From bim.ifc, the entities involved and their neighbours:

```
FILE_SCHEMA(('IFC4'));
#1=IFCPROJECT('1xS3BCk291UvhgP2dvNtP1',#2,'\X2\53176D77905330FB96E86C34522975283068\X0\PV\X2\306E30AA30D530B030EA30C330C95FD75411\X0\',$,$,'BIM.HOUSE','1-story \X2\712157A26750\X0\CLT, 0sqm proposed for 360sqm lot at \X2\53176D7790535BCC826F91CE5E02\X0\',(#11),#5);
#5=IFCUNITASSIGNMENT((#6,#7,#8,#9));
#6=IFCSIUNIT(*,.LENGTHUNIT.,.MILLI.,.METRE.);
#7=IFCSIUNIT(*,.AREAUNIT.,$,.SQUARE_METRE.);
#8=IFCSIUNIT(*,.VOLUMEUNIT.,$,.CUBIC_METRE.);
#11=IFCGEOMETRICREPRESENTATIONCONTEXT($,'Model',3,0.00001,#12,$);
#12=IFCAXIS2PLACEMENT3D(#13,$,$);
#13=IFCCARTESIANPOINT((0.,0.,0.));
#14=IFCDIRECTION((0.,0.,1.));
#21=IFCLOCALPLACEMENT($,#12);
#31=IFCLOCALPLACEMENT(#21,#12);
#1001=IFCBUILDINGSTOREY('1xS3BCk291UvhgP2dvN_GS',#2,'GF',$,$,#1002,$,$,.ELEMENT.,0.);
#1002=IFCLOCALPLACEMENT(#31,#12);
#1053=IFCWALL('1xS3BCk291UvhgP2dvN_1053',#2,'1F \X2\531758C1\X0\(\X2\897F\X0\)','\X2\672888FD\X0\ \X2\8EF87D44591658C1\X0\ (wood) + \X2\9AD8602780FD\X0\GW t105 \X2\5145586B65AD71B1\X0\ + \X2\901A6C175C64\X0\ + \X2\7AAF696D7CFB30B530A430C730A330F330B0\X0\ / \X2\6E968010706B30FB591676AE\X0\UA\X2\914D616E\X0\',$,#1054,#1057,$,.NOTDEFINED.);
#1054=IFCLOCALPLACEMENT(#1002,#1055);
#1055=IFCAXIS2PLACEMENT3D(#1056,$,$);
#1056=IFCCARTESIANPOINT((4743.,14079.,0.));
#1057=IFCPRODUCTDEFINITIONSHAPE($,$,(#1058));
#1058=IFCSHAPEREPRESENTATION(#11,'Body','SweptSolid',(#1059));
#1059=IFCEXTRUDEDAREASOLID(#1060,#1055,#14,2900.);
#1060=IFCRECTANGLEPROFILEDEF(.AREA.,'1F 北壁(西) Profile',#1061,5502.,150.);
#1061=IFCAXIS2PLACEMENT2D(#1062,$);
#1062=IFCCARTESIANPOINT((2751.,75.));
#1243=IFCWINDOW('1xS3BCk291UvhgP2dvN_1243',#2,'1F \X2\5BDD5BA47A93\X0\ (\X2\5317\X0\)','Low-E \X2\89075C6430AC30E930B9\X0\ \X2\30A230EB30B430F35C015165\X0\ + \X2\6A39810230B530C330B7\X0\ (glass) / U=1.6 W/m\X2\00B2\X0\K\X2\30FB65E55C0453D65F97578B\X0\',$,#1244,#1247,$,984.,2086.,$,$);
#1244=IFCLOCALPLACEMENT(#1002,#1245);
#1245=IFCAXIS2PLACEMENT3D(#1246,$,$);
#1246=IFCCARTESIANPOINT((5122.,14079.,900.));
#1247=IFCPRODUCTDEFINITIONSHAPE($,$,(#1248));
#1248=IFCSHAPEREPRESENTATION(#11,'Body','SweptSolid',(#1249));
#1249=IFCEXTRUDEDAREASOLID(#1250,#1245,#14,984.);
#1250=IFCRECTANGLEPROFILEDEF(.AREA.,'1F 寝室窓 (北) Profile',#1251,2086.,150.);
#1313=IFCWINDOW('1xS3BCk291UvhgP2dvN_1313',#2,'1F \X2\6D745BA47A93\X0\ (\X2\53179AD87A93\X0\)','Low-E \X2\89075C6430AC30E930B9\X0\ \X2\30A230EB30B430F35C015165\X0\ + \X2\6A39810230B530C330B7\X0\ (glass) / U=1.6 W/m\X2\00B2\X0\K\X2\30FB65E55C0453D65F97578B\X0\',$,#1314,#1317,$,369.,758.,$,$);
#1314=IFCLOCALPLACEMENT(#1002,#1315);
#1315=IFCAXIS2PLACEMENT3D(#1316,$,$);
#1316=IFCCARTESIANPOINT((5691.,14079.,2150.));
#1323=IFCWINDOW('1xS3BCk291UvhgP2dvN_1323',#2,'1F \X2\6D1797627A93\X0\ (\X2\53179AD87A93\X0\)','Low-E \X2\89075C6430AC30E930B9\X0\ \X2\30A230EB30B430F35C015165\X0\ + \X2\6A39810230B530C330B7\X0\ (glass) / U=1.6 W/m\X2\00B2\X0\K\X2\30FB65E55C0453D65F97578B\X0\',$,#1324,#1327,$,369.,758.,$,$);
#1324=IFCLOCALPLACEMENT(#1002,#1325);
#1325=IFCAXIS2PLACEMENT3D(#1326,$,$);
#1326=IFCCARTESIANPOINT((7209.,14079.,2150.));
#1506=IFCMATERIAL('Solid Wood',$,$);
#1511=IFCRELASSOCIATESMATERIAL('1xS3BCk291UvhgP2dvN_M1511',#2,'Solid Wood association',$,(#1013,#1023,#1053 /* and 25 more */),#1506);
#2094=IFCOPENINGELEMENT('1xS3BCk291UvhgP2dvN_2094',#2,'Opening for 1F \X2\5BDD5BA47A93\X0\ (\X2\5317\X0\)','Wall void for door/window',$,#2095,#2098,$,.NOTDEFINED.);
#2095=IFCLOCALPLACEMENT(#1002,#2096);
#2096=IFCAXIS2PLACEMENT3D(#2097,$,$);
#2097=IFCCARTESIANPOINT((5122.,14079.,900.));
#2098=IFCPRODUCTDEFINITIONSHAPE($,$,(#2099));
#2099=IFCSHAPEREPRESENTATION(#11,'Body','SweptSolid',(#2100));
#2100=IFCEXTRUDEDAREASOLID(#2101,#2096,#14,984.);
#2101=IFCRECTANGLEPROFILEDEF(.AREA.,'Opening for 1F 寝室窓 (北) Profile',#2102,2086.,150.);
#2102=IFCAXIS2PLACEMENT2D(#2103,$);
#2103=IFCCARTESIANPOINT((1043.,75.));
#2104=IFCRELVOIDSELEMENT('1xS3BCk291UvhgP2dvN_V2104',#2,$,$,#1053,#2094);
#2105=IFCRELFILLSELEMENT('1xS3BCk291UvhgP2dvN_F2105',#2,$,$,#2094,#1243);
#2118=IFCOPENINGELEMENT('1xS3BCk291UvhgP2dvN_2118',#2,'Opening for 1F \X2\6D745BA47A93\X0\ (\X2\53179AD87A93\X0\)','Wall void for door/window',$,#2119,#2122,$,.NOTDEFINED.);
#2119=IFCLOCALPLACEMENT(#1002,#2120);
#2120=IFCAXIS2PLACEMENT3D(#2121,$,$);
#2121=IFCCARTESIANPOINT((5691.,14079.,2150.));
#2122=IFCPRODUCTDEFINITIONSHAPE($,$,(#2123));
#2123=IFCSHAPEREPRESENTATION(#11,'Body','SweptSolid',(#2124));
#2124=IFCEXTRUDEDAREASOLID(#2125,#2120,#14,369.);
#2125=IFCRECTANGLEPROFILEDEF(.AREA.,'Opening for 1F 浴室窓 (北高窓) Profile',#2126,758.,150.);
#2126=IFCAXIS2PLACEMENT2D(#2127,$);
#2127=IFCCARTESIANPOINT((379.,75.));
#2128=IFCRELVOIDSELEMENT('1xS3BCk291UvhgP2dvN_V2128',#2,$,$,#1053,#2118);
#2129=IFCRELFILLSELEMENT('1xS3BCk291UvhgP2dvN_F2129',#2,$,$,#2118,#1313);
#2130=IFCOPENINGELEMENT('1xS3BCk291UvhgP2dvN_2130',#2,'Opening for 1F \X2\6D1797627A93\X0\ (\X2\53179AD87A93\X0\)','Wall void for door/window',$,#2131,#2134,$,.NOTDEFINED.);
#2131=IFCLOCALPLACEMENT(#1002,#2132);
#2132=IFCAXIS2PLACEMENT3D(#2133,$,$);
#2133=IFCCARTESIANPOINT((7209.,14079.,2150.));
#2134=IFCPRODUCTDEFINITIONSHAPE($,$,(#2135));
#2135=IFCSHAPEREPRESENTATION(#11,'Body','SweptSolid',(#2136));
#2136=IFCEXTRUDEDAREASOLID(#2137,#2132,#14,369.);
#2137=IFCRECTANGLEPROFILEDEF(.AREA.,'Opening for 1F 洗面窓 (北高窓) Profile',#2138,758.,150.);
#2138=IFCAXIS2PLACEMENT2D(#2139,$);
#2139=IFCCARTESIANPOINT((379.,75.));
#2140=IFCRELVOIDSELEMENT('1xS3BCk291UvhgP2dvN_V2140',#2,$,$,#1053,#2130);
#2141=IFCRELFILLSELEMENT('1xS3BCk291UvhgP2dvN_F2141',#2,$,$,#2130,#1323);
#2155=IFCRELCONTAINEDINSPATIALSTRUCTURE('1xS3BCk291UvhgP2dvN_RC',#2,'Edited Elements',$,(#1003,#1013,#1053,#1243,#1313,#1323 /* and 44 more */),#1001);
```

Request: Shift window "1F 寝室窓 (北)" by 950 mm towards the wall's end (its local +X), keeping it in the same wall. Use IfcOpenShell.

```python
import ifcopenshell
import ifcopenshell.api.geometry
import ifcopenshell.util.placement

model = ifcopenshell.open("bim.ifc")

window = model.by_guid("1xS3BCk291UvhgP2dvN_1243")
opening = window.FillsVoids[0].RelatingOpeningElement
wall = opening.VoidsElements[0].RelatingBuildingElement

wall_matrix = ifcopenshell.util.placement.get_local_placement(wall.ObjectPlacement)
shift = wall_matrix[:3, 0] * 950.0
before = ifcopenshell.util.placement.get_local_placement(window.ObjectPlacement)[:3, 3].copy()

# The window is not placed relative to its opening, so move both.
for product in (opening, window):
    matrix = ifcopenshell.util.placement.get_local_placement(product.ObjectPlacement)
    matrix[:3, 3] += shift
    ifcopenshell.api.geometry.edit_object_placement(model, product=product, matrix=matrix, is_si=False)

after = ifcopenshell.util.placement.get_local_placement(window.ObjectPlacement)[:3, 3]
print("window moved by", (after - before).round(3) + 0.0)

model.write("bim_updated.ifc")
```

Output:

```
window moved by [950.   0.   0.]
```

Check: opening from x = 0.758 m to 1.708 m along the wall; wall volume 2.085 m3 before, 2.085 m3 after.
